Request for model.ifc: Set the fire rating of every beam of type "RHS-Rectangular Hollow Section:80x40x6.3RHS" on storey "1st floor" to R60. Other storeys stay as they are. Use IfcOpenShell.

First a look at what the model holds.

```python
import ifcopenshell
import ifcopenshell.util.element

model = ifcopenshell.open("model.ifc")
print(model.schema)
storey = next(s for s in model.by_type("IfcBuildingStorey") if s.Name == "1st floor")
beams = [e for e in ifcopenshell.util.element.get_decomposition(storey) if e.is_a("IfcBeam")]
seen = {}
for e in beams:
    element_type = ifcopenshell.util.element.get_type(e)
    key = (element_type.Name if element_type != e and element_type else None, ifcopenshell.util.element.get_pset(e, "Pset_BeamCommon", "FireRating"))
    seen[key] = seen.get(key, 0) + 1
for (name, value), count in sorted(seen.items(), key=str):
    print(count, "x", name, "|", value)
```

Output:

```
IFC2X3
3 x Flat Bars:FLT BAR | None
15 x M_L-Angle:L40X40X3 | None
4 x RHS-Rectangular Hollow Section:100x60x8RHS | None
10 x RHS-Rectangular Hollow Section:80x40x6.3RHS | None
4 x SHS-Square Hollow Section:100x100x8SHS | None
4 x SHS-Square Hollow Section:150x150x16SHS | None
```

```python
import ifcopenshell
import ifcopenshell.api.pset
import ifcopenshell.util.element

model = ifcopenshell.open("model.ifc")

storey = next(s for s in model.by_type("IfcBuildingStorey") if s.Name == "1st floor")
beams = [e for e in ifcopenshell.util.element.get_decomposition(storey) if e.is_a("IfcBeam")]

count = 0
for e in beams:
    element_type = ifcopenshell.util.element.get_type(e)
    if element_type in (None, e) or element_type.Name != "RHS-Rectangular Hollow Section:80x40x6.3RHS":
        continue
    # add_pset returns the element's existing set when there is one.
    pset = ifcopenshell.api.pset.add_pset(model, product=e, name="Pset_BeamCommon")
    ifcopenshell.api.pset.edit_pset(model, pset=pset, properties={"FireRating": "R60"})
    count += 1

print(count, "beams updated")

model.write("model_updated.ifc")
```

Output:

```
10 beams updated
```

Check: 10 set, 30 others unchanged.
